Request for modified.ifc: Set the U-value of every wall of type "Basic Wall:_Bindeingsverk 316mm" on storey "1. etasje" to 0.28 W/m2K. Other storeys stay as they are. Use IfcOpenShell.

First a look at what the model holds.

```python
import ifcopenshell
import ifcopenshell.util.element

model = ifcopenshell.open("modified.ifc")
print(model.schema)
storey = next(s for s in model.by_type("IfcBuildingStorey") if s.Name == "1. etasje")
walls = [e for e in ifcopenshell.util.element.get_decomposition(storey) if e.is_a("IfcWall")]
seen = {}
for e in walls:
    element_type = ifcopenshell.util.element.get_type(e)
    key = (element_type.Name if element_type != e and element_type else None, ifcopenshell.util.element.get_pset(e, "Pset_WallCommon", "ThermalTransmittance"))
    seen[key] = seen.get(key, 0) + 1
for (name, value), count in sorted(seen.items(), key=str):
    print(count, "x", name, "|", value)
```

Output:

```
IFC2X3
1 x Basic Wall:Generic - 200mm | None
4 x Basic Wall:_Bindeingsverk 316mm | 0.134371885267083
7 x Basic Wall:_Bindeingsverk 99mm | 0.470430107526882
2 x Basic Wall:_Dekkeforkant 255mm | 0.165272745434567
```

```python
import ifcopenshell
import ifcopenshell.api.pset
import ifcopenshell.util.element

model = ifcopenshell.open("modified.ifc")

storey = next(s for s in model.by_type("IfcBuildingStorey") if s.Name == "1. etasje")
walls = [e for e in ifcopenshell.util.element.get_decomposition(storey) if e.is_a("IfcWall")]

count = 0
for e in walls:
    element_type = ifcopenshell.util.element.get_type(e)
    if element_type in (None, e) or element_type.Name != "Basic Wall:_Bindeingsverk 316mm":
        continue
    # add_pset returns the element's existing set when there is one.
    pset = ifcopenshell.api.pset.add_pset(model, product=e, name="Pset_WallCommon")
    ifcopenshell.api.pset.edit_pset(model, pset=pset, properties={"ThermalTransmittance": 0.28})
    count += 1

print(count, "walls updated")

model.write("modified_updated.ifc")
```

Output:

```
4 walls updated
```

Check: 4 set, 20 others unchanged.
